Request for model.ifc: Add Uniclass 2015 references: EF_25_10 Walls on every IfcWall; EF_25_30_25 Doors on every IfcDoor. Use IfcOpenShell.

First a look at what the model holds.

```python
import ifcopenshell

model = ifcopenshell.open("model.ifc")
print(model.schema)
print("classifications:", [c.Name for c in model.by_type("IfcClassification")])
for ifc_class in ("IfcDoor", "IfcRoof", "IfcStair", "IfcWall", "IfcWindow"):
    print(ifc_class, len(model.by_type(ifc_class)))
```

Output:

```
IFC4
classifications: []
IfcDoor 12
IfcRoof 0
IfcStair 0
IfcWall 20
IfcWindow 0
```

```python
import ifcopenshell
import ifcopenshell.api.classification

model = ifcopenshell.open("model.ifc")

system = ifcopenshell.api.classification.add_classification(model, classification="Uniclass 2015")

codes = {
    "IfcWall": ("EF_25_10", "Walls"),
    "IfcDoor": ("EF_25_30_25", "Doors"),
}
for ifc_class, (code, name) in codes.items():
    products = model.by_type(ifc_class)
    ifcopenshell.api.classification.add_reference(
        model, products=products, classification=system, identification=code, name=name
    )
    print(code, len(products))

model.write("model_rev.ifc")
```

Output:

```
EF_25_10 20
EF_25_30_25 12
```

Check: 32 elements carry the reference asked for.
